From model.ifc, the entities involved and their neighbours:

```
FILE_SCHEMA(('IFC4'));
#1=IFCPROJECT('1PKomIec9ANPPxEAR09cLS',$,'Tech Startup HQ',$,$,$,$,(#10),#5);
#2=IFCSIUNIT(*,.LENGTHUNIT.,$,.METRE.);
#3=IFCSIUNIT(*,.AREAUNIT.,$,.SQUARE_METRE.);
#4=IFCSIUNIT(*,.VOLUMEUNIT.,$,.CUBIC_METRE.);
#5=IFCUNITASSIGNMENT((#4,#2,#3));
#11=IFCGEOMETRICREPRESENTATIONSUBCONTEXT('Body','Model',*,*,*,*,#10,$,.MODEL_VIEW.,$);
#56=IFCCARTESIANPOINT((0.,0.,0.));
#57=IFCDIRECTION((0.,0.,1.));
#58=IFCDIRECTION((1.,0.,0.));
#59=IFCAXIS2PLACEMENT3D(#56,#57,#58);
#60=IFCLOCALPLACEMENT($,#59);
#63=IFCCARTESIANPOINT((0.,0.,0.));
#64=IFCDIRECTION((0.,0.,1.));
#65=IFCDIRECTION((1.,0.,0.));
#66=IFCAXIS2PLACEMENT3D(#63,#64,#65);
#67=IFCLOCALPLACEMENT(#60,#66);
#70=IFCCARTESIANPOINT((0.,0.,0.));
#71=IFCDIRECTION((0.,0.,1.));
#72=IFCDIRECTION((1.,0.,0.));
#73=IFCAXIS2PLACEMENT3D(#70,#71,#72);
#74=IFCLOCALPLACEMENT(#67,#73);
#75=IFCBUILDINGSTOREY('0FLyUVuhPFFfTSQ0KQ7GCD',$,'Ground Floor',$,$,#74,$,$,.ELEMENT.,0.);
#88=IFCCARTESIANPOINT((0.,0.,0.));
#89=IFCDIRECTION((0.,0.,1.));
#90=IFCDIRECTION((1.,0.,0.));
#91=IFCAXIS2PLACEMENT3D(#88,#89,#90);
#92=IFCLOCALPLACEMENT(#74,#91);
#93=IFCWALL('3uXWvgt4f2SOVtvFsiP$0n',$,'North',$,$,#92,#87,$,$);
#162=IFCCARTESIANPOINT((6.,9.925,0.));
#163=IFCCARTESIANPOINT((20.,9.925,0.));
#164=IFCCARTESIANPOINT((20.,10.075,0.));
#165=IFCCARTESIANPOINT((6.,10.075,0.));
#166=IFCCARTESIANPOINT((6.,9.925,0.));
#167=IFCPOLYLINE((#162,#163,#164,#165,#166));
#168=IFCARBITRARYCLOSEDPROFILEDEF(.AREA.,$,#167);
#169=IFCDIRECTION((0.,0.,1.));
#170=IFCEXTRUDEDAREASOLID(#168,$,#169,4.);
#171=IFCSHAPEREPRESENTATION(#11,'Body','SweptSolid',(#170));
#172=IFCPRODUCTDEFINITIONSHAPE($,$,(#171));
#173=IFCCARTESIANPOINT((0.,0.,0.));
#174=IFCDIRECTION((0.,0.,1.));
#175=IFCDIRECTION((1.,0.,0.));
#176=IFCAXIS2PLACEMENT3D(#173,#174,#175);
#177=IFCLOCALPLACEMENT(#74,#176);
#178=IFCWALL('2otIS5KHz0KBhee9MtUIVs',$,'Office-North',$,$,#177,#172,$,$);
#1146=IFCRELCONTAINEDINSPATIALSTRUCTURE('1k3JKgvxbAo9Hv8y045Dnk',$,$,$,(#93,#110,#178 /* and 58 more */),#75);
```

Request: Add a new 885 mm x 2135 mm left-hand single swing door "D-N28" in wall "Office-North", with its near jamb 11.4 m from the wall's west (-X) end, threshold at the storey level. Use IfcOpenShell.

```python
import numpy as np
import ifcopenshell
import ifcopenshell.api.feature
import ifcopenshell.api.geometry
import ifcopenshell.api.root
import ifcopenshell.api.spatial
import ifcopenshell.geom
import ifcopenshell.util.element
import ifcopenshell.util.placement
import ifcopenshell.util.representation
import ifcopenshell.util.shape
import ifcopenshell.util.unit

model = ifcopenshell.open("model.ifc")
unit_scale = ifcopenshell.util.unit.calculate_unit_scale(model)
settings = ifcopenshell.geom.settings()


def volume(element):
    """Net volume in cubic metres, openings subtracted."""
    shape = ifcopenshell.geom.create_shape(settings, element)
    return ifcopenshell.util.shape.get_volume(shape.geometry)


wall = model.by_guid("2otIS5KHz0KBhee9MtUIVs")
storey = ifcopenshell.util.element.get_container(wall, ifc_class="IfcBuildingStorey")
context = ifcopenshell.util.representation.get_context(model, "Model", "Body", "MODEL_VIEW")
before = volume(wall)

width, height, from_end, sill = 0.885, 2.135, 11.4, 0.0  # metres

# The wall runs along its own X axis, and the end named is its -X end.
wall_shape = ifcopenshell.geom.create_shape(settings, wall)
x, y, z = ifcopenshell.util.shape.get_vertices(wall_shape.geometry).T
start = x.min() + from_end
face, thickness = float(y.min()), float(y.max() - y.min())
wall_matrix = ifcopenshell.util.placement.get_local_placement(wall.ObjectPlacement)
level = ifcopenshell.util.placement.get_local_placement(storey.ObjectPlacement)[2, 3]


def in_wall(x, y):
    """Placement at x, y metres in the wall's axes, at sill height."""
    matrix = wall_matrix.copy()
    matrix[:, 3] = wall_matrix @ np.array([x / unit_scale, y / unit_scale, 0.0, 1.0])
    matrix[2, 3] = level + sill / unit_scale
    return matrix


# Opening: a box that overshoots both wall faces by 50 mm.
opening = ifcopenshell.api.root.create_entity(model, ifc_class="IfcOpeningElement", predefined_type="OPENING")
box = ifcopenshell.api.geometry.add_wall_representation(
    model, context=context, length=width, height=height, thickness=thickness + 0.1
)
ifcopenshell.api.geometry.assign_representation(model, product=opening, representation=box)
ifcopenshell.api.geometry.edit_object_placement(model, product=opening, matrix=in_wall(start, face - 0.05), is_si=False)
ifcopenshell.api.feature.add_feature(model, feature=opening, element=wall)

door = ifcopenshell.api.root.create_entity(model, ifc_class="IfcDoor", name="D-N28", predefined_type="DOOR")
door.OverallWidth, door.OverallHeight = width / unit_scale, height / unit_scale
door.OperationType = "SINGLE_SWING_LEFT"
body = ifcopenshell.api.geometry.add_door_representation(
    model,
    context=context,
    overall_width=door.OverallWidth,
    overall_height=door.OverallHeight,
    operation_type="SINGLE_SWING_LEFT",
    lining_properties={"LiningDepth": thickness / unit_scale, "ThresholdDepth": thickness / unit_scale},
)
ifcopenshell.api.geometry.assign_representation(model, product=door, representation=body)
ifcopenshell.api.spatial.assign_container(model, products=[door], relating_structure=storey)
ifcopenshell.api.feature.add_filling(model, opening=opening, element=door)

# The lining spans the wall, so the door starts at the wall face.
ifcopenshell.api.geometry.edit_object_placement(model, product=door, matrix=in_wall(start, face), is_si=False)

after = volume(wall)

print(f"wall volume {before:.3f} -> {after:.3f} m3")

model.write("model-out.ifc")
```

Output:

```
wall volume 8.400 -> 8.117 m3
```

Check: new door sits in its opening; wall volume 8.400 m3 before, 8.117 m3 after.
